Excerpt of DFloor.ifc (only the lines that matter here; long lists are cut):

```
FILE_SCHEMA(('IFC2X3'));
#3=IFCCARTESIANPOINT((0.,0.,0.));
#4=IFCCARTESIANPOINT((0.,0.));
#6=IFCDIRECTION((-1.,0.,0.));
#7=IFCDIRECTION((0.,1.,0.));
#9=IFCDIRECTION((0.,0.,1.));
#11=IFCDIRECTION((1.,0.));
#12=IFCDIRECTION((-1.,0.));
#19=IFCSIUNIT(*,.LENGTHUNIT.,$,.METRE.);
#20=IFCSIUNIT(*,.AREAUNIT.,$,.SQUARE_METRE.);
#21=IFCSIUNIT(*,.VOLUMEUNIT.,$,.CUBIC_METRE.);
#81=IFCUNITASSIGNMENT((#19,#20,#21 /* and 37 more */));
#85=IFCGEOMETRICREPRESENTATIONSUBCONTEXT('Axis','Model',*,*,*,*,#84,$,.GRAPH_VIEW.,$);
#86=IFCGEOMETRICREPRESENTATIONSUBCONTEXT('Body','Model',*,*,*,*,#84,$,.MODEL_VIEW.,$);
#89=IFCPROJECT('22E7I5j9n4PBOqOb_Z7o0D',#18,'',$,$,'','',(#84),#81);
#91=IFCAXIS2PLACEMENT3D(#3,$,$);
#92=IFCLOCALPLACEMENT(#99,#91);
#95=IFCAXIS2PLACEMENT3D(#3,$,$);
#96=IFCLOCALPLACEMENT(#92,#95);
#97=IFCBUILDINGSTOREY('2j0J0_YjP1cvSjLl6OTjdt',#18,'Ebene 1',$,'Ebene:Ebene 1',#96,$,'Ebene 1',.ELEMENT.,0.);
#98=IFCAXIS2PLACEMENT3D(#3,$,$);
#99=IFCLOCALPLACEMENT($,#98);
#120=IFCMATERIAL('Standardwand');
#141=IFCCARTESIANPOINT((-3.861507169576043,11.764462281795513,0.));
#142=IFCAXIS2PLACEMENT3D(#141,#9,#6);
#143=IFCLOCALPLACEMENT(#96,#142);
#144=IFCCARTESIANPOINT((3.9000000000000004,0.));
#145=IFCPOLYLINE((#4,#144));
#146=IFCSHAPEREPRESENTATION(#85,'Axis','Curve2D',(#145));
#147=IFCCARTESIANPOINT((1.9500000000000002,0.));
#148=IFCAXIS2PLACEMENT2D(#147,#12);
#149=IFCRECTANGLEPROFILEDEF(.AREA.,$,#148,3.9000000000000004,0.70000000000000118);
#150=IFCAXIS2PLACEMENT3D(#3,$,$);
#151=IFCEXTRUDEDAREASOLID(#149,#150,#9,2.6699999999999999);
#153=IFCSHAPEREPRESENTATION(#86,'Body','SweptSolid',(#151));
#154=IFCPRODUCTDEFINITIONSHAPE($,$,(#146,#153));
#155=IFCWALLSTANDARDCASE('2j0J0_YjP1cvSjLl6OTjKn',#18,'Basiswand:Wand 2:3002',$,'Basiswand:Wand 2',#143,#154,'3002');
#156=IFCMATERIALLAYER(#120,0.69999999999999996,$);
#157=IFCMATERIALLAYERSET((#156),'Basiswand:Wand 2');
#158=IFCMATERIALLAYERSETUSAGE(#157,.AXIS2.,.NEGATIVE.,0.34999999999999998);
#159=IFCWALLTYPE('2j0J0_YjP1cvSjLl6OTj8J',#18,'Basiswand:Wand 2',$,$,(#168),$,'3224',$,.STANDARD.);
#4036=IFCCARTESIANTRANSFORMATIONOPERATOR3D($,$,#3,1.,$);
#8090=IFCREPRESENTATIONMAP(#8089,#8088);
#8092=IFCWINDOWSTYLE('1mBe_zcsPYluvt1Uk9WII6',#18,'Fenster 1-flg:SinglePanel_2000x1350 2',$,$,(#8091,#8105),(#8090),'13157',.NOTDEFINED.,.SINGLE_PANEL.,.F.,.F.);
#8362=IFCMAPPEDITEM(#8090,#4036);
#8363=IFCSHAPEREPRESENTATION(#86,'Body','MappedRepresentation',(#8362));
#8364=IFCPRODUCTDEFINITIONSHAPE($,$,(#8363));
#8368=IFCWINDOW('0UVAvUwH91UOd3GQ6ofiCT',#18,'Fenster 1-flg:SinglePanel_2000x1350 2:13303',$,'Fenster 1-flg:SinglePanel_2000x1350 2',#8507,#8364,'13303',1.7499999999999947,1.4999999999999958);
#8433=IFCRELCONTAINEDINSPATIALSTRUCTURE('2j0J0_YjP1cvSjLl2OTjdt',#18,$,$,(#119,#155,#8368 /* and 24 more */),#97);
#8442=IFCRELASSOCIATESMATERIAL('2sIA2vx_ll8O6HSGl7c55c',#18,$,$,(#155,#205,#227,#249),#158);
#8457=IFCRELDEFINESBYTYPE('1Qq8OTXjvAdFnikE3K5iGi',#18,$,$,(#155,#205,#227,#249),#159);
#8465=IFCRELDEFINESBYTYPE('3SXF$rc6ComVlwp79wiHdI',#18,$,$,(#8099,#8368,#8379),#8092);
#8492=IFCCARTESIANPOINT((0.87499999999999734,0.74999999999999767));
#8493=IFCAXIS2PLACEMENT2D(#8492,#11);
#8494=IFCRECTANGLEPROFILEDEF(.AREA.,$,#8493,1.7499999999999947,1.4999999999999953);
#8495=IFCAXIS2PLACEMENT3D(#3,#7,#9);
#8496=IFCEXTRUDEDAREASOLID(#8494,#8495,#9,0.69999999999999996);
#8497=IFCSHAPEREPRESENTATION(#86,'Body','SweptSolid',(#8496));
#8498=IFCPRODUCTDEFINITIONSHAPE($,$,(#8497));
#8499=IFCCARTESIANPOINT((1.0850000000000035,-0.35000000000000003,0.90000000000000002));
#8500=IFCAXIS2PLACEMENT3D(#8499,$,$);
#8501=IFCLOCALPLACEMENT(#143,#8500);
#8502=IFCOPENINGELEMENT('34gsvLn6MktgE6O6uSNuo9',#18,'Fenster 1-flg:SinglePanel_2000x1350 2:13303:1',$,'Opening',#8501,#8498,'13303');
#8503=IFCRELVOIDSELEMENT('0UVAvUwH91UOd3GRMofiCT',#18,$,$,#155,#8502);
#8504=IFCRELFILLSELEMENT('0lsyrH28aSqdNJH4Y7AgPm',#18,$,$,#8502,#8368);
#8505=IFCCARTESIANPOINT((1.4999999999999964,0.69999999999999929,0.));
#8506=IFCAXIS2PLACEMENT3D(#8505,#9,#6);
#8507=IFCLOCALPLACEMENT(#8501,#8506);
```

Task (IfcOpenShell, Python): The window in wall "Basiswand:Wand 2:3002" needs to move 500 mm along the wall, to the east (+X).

```python
import ifcopenshell
import ifcopenshell.api.geometry
import ifcopenshell.util.placement

model = ifcopenshell.open("DFloor.ifc")

window = model.by_guid("0UVAvUwH91UOd3GQ6ofiCT")
opening = window.FillsVoids[0].RelatingOpeningElement
wall = opening.VoidsElements[0].RelatingBuildingElement

wall_matrix = ifcopenshell.util.placement.get_local_placement(wall.ObjectPlacement)
shift = wall_matrix[:3, 0] * -0.5
before = ifcopenshell.util.placement.get_local_placement(window.ObjectPlacement)[:3, 3].copy()

# The window is placed relative to its opening, so it follows when the opening moves.
matrix = ifcopenshell.util.placement.get_local_placement(opening.ObjectPlacement)
matrix[:3, 3] += shift
ifcopenshell.api.geometry.edit_object_placement(
    model, product=opening, matrix=matrix, is_si=False, should_transform_children=True
)

after = ifcopenshell.util.placement.get_local_placement(window.ObjectPlacement)[:3, 3]
print("window moved by", (after - before).round(3) + 0.0)

model.write("DFloor_updated.ifc")
```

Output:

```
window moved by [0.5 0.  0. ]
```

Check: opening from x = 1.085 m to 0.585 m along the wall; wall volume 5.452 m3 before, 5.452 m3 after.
